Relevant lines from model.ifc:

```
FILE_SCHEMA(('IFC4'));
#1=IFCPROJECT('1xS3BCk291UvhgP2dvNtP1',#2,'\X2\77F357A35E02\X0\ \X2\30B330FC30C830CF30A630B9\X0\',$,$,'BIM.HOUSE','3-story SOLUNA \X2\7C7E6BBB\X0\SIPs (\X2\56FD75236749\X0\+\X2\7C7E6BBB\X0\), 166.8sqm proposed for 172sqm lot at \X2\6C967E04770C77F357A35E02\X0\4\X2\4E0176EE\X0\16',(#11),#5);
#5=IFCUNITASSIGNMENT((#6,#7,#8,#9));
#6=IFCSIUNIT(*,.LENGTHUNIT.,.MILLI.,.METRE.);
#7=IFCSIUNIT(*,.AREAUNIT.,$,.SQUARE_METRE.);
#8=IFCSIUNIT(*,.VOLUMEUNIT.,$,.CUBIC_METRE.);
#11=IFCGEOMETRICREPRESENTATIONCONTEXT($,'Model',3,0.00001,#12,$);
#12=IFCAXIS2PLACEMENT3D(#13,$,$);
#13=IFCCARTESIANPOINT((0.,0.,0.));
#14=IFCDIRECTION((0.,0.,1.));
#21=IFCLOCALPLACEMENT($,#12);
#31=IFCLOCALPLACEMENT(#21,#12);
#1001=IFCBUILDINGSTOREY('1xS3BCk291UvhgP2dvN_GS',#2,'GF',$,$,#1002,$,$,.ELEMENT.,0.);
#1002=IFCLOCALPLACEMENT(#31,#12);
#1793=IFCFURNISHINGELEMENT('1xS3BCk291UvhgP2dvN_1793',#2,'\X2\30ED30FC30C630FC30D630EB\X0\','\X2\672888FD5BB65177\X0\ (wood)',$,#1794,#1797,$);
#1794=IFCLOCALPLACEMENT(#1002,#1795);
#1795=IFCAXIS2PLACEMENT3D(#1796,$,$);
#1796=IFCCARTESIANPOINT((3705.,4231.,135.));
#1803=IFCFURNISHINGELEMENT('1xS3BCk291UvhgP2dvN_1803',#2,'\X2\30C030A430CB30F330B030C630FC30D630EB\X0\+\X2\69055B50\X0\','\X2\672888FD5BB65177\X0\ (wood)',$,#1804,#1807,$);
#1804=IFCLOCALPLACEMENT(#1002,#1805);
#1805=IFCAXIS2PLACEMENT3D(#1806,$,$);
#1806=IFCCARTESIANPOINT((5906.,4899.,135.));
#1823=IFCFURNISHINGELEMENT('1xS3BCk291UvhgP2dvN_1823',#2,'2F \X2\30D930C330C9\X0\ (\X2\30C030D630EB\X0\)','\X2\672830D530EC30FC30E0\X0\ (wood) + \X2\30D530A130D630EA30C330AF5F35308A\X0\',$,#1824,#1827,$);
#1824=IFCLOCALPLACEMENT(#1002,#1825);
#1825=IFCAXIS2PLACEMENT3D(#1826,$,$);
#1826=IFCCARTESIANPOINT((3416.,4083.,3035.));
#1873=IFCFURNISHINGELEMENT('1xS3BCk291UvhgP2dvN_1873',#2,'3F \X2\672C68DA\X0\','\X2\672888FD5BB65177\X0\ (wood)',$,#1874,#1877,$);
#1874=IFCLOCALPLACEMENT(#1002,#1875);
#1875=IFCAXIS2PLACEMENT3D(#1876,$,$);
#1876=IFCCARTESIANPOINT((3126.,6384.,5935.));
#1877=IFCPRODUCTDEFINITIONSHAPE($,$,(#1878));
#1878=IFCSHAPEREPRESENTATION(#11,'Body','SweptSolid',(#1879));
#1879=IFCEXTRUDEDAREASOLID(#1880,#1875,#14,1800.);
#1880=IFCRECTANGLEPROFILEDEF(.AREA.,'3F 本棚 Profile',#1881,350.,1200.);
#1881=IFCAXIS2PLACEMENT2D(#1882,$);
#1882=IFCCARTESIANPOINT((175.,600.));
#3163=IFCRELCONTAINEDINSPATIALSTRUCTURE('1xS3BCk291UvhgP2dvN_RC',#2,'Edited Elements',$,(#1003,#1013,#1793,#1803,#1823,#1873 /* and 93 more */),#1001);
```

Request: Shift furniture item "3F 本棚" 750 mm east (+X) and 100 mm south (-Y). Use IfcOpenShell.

```python
import ifcopenshell
import ifcopenshell.api.geometry
import ifcopenshell.util.placement

model = ifcopenshell.open("model.ifc")

item = model.by_guid("1xS3BCk291UvhgP2dvN_1873")
matrix = ifcopenshell.util.placement.get_local_placement(item.ObjectPlacement)
matrix[0, 3] += 750.0
matrix[1, 3] -= 100.0
ifcopenshell.api.geometry.edit_object_placement(model, product=item, matrix=matrix, is_si=False)

print(ifcopenshell.util.placement.get_local_placement(item.ObjectPlacement).round(3) + 0.0)

model.write("model_rev.ifc")
```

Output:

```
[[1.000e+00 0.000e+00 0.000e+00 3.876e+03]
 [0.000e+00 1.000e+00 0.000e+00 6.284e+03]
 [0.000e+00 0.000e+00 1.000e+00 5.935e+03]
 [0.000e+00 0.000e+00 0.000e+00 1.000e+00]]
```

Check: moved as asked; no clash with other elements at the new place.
